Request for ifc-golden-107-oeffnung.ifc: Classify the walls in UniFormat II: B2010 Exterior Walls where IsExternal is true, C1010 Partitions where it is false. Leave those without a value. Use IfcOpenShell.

First a look at what the model holds.

```python
import ifcopenshell
import ifcopenshell.util.element

model = ifcopenshell.open("ifc-golden-107-oeffnung.ifc")
print(model.schema)
print("classifications:", [c.Name for c in model.by_type("IfcClassification")])
values = [ifcopenshell.util.element.get_pset(e, "Pset_WallCommon", "IsExternal") for e in model.by_type("IfcWall")]
for value in (True, False, None):
    print("IsExternal", value, values.count(value))
```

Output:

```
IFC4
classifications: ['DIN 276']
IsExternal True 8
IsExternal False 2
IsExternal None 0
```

```python
import ifcopenshell
import ifcopenshell.api.classification
import ifcopenshell.util.element

model = ifcopenshell.open("ifc-golden-107-oeffnung.ifc")

system = ifcopenshell.api.classification.add_classification(model, classification="UniFormat II")

walls = model.by_type("IfcWall")
external = {e: ifcopenshell.util.element.get_pset(e, "Pset_WallCommon", "IsExternal") for e in walls}
for flag, code, name in ((True, "B2010", "Exterior Walls"), (False, "C1010", "Partitions")):
    products = [e for e in walls if external[e] is flag]
    ifcopenshell.api.classification.add_reference(
        model, products=products, classification=system, identification=code, name=name
    )
    print(code, len(products))

model.write("ifc-golden-107-oeffnung-out.ifc")
```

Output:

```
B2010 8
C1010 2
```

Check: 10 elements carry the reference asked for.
